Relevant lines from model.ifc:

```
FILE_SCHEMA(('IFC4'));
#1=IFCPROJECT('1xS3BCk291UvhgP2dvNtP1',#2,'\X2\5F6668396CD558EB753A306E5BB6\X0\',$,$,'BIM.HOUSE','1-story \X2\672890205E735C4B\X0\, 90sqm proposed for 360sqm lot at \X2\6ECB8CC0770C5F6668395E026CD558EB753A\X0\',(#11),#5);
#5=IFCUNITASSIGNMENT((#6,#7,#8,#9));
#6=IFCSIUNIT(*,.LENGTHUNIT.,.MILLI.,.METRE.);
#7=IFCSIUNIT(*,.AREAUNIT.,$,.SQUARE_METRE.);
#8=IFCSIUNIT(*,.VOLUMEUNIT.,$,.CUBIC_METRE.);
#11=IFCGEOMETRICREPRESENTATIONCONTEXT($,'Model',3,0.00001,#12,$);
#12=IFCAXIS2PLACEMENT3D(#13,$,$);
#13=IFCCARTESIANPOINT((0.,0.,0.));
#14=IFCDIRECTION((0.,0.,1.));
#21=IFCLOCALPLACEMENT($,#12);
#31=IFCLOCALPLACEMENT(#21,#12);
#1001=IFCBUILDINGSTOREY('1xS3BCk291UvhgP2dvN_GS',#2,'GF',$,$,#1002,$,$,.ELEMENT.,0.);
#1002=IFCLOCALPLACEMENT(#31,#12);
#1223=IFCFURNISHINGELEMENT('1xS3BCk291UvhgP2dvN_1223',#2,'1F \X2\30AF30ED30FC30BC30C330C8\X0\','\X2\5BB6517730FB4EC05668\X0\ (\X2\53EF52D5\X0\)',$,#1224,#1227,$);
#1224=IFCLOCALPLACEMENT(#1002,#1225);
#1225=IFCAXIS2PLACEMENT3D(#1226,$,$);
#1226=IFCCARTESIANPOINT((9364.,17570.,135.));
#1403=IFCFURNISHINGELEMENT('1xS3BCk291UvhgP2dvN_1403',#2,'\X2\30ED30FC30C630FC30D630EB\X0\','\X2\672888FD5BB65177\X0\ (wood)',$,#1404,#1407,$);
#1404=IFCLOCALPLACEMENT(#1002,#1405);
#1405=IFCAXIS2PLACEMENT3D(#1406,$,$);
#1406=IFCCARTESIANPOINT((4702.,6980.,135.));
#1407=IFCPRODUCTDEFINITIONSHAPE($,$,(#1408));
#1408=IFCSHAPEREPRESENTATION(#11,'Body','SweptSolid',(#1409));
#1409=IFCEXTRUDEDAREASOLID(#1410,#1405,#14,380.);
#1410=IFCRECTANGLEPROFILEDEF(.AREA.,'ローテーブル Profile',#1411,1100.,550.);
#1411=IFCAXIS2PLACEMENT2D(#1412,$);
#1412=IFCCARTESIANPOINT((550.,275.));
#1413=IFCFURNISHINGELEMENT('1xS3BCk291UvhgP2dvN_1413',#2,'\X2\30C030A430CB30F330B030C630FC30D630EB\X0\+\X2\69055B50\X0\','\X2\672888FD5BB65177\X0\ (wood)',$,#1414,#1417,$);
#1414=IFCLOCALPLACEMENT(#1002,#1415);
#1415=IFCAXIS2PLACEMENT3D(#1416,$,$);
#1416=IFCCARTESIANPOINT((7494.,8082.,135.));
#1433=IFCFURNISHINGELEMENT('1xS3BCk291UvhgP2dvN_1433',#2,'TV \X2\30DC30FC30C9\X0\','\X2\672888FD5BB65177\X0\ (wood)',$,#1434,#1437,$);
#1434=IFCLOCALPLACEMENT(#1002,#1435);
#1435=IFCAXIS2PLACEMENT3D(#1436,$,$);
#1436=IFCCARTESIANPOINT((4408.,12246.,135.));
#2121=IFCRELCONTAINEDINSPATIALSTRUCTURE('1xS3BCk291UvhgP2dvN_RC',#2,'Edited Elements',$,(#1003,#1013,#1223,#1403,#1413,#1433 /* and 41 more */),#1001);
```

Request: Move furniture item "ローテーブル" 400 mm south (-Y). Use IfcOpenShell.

```python
import ifcopenshell
import ifcopenshell.api.geometry
import ifcopenshell.util.placement
import ifcopenshell.util.unit

model = ifcopenshell.open("model.ifc")
unit_scale = ifcopenshell.util.unit.calculate_unit_scale(model)

item = model.by_guid("1xS3BCk291UvhgP2dvN_1403")
matrix = ifcopenshell.util.placement.get_local_placement(item.ObjectPlacement)
matrix[1, 3] -= 0.4 / unit_scale
ifcopenshell.api.geometry.edit_object_placement(model, product=item, matrix=matrix, is_si=False)

print(ifcopenshell.util.placement.get_local_placement(item.ObjectPlacement).round(3) + 0.0)

model.write("model-out.ifc")
```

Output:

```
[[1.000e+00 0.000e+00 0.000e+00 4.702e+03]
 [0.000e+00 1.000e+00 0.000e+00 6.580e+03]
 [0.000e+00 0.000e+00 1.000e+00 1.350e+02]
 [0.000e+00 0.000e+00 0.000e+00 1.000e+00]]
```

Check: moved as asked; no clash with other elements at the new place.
